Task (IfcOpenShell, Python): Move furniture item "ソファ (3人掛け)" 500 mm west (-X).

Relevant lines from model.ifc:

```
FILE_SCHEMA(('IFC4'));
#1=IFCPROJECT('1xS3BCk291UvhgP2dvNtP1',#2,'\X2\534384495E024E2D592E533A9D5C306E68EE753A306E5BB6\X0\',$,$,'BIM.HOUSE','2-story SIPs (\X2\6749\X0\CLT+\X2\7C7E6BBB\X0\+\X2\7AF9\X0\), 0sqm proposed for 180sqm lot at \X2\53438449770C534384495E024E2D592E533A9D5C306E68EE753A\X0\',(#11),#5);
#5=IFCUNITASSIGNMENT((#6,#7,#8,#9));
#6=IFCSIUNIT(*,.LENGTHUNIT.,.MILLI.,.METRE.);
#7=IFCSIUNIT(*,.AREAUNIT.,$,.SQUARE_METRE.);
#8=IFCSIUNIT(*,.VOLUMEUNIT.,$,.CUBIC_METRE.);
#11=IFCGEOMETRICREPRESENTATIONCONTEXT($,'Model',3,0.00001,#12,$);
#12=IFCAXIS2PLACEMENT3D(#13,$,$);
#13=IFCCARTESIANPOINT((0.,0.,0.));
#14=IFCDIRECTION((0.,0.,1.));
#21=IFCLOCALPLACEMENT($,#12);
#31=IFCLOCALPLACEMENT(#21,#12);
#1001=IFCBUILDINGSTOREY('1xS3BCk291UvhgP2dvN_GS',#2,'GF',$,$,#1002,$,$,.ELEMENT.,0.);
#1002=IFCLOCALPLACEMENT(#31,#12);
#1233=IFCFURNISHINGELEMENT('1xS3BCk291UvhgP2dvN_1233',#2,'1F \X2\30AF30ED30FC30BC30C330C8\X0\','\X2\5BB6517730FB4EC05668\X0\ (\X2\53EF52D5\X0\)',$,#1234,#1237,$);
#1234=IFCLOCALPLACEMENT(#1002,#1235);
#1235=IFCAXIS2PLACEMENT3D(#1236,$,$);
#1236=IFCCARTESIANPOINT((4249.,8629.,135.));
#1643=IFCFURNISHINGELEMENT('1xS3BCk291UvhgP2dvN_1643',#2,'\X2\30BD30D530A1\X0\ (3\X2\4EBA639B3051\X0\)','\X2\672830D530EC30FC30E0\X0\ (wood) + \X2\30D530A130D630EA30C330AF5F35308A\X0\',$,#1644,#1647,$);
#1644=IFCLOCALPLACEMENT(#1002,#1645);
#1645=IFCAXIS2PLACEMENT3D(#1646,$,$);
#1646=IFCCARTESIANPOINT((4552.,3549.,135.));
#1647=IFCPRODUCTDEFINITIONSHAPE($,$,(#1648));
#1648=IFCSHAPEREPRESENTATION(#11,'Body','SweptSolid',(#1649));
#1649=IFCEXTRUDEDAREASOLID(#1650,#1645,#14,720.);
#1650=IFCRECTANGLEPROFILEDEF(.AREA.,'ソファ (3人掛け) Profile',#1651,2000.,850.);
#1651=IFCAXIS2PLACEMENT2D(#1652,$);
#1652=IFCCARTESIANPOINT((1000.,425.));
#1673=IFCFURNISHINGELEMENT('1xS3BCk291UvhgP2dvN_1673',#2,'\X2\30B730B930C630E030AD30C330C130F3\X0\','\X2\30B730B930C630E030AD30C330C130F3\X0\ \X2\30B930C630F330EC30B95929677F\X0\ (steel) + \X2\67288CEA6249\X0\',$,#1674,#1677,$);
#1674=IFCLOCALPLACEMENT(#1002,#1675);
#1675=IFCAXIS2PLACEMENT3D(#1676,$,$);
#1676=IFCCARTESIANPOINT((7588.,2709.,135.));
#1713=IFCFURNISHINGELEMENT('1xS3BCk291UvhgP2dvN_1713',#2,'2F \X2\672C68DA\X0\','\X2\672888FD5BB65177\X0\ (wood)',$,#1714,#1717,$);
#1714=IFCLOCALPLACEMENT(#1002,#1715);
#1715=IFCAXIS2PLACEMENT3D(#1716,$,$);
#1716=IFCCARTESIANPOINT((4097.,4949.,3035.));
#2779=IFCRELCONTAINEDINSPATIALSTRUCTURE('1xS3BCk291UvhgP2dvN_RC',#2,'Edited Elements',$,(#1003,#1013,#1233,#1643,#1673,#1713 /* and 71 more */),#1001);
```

```python
import ifcopenshell
import ifcopenshell.api.geometry
import ifcopenshell.util.placement
import ifcopenshell.util.unit

model = ifcopenshell.open("model.ifc")
unit_scale = ifcopenshell.util.unit.calculate_unit_scale(model)

item = model.by_guid("1xS3BCk291UvhgP2dvN_1643")
matrix = ifcopenshell.util.placement.get_local_placement(item.ObjectPlacement)
matrix[0, 3] -= 0.5 / unit_scale
ifcopenshell.api.geometry.edit_object_placement(model, product=item, matrix=matrix, is_si=False)

print(ifcopenshell.util.placement.get_local_placement(item.ObjectPlacement).round(3) + 0.0)

model.write("model_v2.ifc")
```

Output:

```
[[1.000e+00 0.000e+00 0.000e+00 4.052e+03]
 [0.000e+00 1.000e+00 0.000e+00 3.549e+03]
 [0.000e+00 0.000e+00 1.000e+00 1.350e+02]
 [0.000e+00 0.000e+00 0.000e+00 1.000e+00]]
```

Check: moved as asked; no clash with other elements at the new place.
